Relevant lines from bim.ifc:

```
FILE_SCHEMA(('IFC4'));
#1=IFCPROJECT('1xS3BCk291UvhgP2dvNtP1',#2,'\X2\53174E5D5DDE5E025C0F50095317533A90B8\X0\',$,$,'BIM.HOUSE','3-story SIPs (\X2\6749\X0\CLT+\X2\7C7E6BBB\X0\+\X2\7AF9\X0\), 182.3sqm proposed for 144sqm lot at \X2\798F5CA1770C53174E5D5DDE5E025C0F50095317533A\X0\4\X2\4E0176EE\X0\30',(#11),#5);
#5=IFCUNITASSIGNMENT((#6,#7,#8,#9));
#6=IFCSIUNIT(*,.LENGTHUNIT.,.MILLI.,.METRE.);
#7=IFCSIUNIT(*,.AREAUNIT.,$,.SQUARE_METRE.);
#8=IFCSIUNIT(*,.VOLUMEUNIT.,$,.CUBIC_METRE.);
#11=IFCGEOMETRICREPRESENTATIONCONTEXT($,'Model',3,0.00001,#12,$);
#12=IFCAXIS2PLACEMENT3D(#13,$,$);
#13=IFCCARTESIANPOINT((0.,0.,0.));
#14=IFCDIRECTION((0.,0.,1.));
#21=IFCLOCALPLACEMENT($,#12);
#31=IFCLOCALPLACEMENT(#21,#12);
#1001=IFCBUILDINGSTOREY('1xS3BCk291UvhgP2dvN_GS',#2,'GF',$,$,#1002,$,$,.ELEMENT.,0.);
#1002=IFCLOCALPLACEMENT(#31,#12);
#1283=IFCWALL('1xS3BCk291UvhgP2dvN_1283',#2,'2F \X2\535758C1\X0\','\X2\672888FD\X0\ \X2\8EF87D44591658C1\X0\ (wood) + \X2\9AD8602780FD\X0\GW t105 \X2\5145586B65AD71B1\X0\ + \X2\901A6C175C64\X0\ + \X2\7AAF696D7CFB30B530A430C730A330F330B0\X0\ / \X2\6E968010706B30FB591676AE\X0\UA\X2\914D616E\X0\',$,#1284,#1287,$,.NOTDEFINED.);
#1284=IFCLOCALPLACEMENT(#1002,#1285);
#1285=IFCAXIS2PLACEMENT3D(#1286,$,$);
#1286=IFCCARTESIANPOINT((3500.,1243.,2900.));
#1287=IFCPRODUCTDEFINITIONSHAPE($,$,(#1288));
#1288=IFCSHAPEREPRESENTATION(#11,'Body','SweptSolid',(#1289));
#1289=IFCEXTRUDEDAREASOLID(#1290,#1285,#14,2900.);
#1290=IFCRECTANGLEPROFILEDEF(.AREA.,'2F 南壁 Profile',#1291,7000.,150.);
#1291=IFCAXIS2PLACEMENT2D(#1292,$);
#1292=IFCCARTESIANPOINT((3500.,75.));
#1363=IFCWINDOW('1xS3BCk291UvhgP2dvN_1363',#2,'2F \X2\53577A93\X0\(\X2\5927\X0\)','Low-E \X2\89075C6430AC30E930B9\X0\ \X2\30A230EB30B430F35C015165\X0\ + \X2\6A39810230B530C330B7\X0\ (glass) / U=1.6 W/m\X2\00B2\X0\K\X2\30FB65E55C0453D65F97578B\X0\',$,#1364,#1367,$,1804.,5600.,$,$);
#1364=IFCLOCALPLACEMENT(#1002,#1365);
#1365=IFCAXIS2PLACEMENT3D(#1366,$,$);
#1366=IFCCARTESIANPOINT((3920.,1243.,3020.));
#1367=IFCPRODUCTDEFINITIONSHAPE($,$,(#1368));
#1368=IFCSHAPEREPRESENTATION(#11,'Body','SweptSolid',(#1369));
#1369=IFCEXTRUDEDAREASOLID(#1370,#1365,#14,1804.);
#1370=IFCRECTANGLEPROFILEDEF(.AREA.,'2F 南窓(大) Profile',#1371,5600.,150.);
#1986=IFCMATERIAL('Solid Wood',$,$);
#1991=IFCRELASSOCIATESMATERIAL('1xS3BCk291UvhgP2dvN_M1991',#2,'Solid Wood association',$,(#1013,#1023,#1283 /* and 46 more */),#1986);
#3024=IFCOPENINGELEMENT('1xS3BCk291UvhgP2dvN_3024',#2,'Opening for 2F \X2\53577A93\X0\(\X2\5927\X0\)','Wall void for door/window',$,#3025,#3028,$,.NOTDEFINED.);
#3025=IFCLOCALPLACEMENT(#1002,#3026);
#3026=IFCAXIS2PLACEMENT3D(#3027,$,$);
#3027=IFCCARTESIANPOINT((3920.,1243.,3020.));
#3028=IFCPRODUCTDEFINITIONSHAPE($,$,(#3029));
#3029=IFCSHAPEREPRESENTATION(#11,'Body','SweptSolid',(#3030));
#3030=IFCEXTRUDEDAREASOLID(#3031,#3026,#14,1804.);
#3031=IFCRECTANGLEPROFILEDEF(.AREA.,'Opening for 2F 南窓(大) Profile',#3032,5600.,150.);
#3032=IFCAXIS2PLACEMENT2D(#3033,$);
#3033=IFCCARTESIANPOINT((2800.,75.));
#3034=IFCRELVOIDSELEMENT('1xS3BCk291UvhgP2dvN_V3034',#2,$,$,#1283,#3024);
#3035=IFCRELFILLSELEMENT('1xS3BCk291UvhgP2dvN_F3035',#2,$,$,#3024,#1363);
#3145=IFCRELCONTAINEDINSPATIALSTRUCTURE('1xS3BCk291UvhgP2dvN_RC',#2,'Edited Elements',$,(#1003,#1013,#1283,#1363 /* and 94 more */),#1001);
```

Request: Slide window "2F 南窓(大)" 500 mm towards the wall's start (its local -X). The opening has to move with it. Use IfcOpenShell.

```python
import ifcopenshell
import ifcopenshell.api.geometry
import ifcopenshell.util.placement
import ifcopenshell.util.unit

model = ifcopenshell.open("bim.ifc")
unit_scale = ifcopenshell.util.unit.calculate_unit_scale(model)

window = model.by_id(1363)
opening = window.FillsVoids[0].RelatingOpeningElement
wall = opening.VoidsElements[0].RelatingBuildingElement

wall_matrix = ifcopenshell.util.placement.get_local_placement(wall.ObjectPlacement)
shift = wall_matrix[:3, 0] * -0.5 / unit_scale
before = ifcopenshell.util.placement.get_local_placement(window.ObjectPlacement)[:3, 3].copy()

# The window is not placed relative to its opening, so move both.
for product in (opening, window):
    matrix = ifcopenshell.util.placement.get_local_placement(product.ObjectPlacement)
    matrix[:3, 3] += shift
    ifcopenshell.api.geometry.edit_object_placement(model, product=product, matrix=matrix, is_si=False)

after = ifcopenshell.util.placement.get_local_placement(window.ObjectPlacement)[:3, 3]
print("window moved by", (after - before).round(3) + 0.0)

model.write("bim-out.ifc")
```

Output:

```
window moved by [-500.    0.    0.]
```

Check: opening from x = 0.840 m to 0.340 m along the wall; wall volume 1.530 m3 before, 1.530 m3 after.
